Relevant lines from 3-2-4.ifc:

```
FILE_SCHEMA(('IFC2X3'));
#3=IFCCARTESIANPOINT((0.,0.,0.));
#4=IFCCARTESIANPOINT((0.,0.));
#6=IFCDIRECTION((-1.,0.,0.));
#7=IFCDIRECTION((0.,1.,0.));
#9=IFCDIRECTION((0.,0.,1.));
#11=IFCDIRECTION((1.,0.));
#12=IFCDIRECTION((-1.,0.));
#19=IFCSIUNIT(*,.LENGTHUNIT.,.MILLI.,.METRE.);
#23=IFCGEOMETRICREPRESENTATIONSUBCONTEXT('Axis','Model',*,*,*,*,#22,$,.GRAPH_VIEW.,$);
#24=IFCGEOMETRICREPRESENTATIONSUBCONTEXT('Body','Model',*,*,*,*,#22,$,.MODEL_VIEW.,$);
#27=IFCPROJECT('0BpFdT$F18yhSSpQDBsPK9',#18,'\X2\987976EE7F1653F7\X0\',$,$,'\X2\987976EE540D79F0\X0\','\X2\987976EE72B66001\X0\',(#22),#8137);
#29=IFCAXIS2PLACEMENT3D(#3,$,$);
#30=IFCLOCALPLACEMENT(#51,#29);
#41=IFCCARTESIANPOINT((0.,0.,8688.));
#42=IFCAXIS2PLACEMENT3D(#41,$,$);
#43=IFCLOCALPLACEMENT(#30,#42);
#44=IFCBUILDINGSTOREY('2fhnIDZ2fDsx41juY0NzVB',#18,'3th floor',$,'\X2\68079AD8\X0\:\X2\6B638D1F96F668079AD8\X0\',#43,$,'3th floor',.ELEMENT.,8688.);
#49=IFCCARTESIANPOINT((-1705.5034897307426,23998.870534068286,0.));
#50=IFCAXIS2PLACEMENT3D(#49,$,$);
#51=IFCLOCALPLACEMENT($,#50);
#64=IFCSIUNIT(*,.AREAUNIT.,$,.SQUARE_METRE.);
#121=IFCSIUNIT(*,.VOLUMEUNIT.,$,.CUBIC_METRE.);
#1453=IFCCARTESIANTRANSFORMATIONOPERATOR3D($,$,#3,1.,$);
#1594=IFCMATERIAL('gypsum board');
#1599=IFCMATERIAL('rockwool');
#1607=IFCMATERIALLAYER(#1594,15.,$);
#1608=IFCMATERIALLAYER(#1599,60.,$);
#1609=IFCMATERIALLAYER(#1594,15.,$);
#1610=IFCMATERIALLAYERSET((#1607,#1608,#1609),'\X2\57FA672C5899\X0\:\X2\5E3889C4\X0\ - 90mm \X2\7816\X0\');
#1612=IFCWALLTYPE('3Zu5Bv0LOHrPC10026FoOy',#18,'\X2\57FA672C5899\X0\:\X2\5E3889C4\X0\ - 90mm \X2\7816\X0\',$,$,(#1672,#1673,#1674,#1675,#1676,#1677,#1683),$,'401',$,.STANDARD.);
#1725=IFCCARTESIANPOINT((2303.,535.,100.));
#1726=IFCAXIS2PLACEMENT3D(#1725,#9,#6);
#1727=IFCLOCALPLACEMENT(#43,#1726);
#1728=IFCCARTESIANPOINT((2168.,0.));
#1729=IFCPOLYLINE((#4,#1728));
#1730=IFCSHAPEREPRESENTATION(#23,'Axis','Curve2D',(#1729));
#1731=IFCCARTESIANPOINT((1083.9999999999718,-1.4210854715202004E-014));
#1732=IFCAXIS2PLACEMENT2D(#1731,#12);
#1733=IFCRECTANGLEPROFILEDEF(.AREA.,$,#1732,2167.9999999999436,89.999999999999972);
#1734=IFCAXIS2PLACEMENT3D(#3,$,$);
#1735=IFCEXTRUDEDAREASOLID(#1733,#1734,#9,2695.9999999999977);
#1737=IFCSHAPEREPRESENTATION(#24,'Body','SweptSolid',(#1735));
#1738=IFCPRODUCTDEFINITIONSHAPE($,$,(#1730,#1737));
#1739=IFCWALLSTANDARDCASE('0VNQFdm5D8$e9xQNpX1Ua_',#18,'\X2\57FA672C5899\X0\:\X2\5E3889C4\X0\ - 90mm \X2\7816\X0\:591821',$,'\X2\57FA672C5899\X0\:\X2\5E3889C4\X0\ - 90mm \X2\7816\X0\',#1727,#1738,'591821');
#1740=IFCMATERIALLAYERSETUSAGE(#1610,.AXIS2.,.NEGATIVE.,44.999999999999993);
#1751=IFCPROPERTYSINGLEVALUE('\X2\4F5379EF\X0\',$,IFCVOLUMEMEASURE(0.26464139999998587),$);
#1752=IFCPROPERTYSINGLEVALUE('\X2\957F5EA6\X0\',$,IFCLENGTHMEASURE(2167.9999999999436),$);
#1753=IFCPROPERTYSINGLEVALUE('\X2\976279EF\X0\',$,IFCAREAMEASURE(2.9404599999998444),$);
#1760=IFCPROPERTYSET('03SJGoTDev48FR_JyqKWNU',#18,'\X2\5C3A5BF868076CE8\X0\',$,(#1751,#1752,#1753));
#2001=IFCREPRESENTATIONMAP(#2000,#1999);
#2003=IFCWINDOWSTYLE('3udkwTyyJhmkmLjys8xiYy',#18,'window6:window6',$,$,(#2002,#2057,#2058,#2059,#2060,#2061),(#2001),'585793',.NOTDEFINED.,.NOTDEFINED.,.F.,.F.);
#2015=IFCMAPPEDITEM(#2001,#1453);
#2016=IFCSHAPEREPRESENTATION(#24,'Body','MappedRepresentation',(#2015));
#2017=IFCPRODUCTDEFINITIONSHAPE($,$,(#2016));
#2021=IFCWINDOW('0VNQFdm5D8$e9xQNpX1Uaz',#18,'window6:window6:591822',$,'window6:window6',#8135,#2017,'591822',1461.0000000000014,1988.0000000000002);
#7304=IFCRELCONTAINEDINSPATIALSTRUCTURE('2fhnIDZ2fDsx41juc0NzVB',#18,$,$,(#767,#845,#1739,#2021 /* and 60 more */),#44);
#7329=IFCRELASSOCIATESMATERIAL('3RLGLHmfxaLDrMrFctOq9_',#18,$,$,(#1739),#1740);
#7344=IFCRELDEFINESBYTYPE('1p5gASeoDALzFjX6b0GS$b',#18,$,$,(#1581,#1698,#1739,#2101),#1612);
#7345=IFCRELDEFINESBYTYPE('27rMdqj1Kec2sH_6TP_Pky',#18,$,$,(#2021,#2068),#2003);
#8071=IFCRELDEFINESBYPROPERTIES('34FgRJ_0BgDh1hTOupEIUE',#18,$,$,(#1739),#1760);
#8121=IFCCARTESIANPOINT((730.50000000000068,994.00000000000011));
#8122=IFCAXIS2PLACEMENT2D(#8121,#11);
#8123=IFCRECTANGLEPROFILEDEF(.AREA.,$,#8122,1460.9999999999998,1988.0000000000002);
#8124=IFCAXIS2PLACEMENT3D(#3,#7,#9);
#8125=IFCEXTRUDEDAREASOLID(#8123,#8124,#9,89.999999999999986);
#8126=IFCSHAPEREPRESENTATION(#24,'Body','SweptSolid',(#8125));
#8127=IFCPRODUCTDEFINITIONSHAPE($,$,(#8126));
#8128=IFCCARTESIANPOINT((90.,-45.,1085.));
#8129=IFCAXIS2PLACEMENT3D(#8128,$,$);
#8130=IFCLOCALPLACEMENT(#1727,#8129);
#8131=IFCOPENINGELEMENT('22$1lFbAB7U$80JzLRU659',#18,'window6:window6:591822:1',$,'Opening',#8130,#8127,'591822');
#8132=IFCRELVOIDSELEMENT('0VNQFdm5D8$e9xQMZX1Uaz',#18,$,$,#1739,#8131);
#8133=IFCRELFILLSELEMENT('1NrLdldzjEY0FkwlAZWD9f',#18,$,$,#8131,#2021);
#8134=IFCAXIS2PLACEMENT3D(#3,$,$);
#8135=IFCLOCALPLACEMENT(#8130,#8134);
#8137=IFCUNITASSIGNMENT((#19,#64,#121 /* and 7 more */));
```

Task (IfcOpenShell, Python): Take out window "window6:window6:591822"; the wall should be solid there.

```python
import ifcopenshell
import ifcopenshell.api.feature
import ifcopenshell.api.pset
import ifcopenshell.api.root
import ifcopenshell.geom
import ifcopenshell.util.element
import ifcopenshell.util.shape
import ifcopenshell.util.unit

model = ifcopenshell.open("3-2-4.ifc")
area_scale = ifcopenshell.util.unit.calculate_unit_scale(model, "AREAUNIT")
volume_scale = ifcopenshell.util.unit.calculate_unit_scale(model, "VOLUMEUNIT")
settings = ifcopenshell.geom.settings()


def volume(element):
    """Net volume in cubic metres, openings subtracted."""
    shape = ifcopenshell.geom.create_shape(settings, element)
    return ifcopenshell.util.shape.get_volume(shape.geometry)


window = model.by_guid("0VNQFdm5D8$e9xQNpX1Uaz")
opening = window.FillsVoids[0].RelatingOpeningElement
wall = opening.VoidsElements[0].RelatingBuildingElement
before = volume(wall)

ifcopenshell.api.root.remove_product(model, product=window)
ifcopenshell.api.feature.remove_feature(model, feature=opening)

after = volume(wall)
thickness = 0.09  # wall thickness in metres

# Update the wall's stored quantities.
pset = model.by_id(ifcopenshell.util.element.get_pset(wall, "尺寸标注", should_inherit=False)["id"])
ifcopenshell.api.pset.edit_pset(model, pset=pset, properties={
    "体积": model.create_entity("IfcVolumeMeasure", after / volume_scale),
    "面积": model.create_entity("IfcAreaMeasure", after / thickness / area_scale),
})

print(f"wall volume {before:.3f} -> {after:.3f} m3")

model.write("3-2-4-out.ifc")
```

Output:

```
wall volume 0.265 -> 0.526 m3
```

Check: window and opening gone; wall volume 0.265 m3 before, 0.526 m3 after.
